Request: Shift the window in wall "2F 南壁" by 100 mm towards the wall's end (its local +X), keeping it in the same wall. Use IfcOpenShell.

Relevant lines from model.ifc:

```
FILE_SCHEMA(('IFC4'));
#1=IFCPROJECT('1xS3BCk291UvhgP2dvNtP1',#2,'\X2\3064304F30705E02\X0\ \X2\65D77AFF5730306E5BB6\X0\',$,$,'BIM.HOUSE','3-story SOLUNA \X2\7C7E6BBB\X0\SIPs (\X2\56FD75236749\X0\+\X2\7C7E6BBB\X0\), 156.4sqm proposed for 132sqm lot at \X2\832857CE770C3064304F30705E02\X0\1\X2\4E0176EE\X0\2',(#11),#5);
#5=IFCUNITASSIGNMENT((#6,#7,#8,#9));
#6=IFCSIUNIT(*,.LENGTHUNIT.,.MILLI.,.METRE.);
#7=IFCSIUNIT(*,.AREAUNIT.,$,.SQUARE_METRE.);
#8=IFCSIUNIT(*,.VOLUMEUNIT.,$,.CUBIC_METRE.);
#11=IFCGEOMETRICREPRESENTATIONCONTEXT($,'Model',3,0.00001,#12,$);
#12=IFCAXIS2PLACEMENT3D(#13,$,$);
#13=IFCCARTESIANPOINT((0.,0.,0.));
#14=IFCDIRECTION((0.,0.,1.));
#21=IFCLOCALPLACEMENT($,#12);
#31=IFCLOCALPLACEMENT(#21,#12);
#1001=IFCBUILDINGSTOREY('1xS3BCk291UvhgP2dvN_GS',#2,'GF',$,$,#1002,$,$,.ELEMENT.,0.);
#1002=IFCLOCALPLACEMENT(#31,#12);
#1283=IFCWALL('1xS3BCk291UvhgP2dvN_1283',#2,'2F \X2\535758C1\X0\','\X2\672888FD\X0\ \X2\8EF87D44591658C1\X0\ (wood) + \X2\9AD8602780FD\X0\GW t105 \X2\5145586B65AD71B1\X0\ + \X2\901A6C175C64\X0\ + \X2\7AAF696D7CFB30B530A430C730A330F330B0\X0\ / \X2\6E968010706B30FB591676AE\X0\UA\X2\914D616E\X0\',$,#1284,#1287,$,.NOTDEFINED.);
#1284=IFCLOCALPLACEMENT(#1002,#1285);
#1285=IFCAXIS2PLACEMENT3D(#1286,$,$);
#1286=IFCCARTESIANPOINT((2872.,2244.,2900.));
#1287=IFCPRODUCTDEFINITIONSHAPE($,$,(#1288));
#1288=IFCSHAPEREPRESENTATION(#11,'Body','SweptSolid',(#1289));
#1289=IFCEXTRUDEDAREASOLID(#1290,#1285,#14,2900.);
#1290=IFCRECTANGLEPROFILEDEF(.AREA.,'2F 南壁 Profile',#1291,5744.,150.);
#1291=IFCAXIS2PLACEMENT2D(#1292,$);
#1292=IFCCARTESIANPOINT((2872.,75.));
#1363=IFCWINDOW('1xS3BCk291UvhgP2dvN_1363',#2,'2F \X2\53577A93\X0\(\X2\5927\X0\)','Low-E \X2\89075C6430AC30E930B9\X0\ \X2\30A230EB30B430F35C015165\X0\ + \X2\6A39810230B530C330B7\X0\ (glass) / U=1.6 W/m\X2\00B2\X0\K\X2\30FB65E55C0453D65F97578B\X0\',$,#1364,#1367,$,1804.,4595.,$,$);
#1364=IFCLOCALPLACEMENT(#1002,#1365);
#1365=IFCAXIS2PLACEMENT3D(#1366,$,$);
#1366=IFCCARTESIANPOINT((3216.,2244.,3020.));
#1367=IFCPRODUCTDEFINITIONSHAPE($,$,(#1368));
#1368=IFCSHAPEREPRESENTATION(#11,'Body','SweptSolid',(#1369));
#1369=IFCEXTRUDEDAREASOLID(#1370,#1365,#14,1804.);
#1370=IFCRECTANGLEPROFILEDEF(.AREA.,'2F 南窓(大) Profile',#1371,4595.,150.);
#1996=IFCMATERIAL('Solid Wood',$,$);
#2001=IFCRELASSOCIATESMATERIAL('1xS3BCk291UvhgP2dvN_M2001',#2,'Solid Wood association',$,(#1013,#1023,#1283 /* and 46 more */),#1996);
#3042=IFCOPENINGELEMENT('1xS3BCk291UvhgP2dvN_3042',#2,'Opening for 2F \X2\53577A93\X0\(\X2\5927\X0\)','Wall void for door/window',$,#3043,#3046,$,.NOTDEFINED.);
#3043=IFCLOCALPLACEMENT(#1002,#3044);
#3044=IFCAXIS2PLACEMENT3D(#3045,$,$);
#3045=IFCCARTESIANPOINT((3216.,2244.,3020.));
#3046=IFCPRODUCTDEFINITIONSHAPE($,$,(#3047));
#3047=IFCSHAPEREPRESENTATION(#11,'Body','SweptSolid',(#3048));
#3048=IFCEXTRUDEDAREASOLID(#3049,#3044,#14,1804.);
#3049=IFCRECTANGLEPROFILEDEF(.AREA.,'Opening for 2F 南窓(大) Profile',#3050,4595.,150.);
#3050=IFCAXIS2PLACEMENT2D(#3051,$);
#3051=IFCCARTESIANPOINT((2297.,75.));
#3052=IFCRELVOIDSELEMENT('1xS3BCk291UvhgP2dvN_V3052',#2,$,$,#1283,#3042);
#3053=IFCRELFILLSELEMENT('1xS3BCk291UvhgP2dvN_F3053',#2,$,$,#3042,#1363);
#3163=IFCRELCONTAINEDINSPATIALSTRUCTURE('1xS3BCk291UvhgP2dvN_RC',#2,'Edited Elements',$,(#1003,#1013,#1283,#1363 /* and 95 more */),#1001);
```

```python
import ifcopenshell
import ifcopenshell.api.geometry
import ifcopenshell.util.placement
import ifcopenshell.util.unit

model = ifcopenshell.open("model.ifc")
unit_scale = ifcopenshell.util.unit.calculate_unit_scale(model)

window = model.by_guid("1xS3BCk291UvhgP2dvN_1363")
opening = window.FillsVoids[0].RelatingOpeningElement
wall = opening.VoidsElements[0].RelatingBuildingElement

wall_matrix = ifcopenshell.util.placement.get_local_placement(wall.ObjectPlacement)
shift = wall_matrix[:3, 0] * 0.1 / unit_scale
before = ifcopenshell.util.placement.get_local_placement(window.ObjectPlacement)[:3, 3].copy()

# The window is not placed relative to its opening, so move both.
for product in (opening, window):
    matrix = ifcopenshell.util.placement.get_local_placement(product.ObjectPlacement)
    matrix[:3, 3] += shift
    ifcopenshell.api.geometry.edit_object_placement(model, product=product, matrix=matrix, is_si=False)

after = ifcopenshell.util.placement.get_local_placement(window.ObjectPlacement)[:3, 3]
print("window moved by", (after - before).round(3) + 0.0)

model.write("model_updated.ifc")
```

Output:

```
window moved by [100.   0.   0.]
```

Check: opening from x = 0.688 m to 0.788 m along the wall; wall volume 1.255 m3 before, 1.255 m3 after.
